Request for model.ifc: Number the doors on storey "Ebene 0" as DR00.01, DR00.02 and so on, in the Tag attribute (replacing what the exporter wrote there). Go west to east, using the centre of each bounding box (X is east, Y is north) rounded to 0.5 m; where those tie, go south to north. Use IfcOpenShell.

First a look at what the model holds.

```python
import ifcopenshell
import ifcopenshell.util.element
import ifcopenshell.util.placement

model = ifcopenshell.open("model.ifc")
print(model.schema)
storey = next(s for s in model.by_type("IfcBuildingStorey") if s.Name == "Ebene 0")
doors = [e for e in ifcopenshell.util.element.get_decomposition(storey) if e.is_a("IfcDoor")]
for e in sorted(doors, key=lambda e: e.id()):
    origin = ifcopenshell.util.placement.get_local_placement(e.ObjectPlacement)[:3, 3]
    print(e.id(), e.Tag, e.Name, origin.round(2) + 0.0, sep=" | ")
```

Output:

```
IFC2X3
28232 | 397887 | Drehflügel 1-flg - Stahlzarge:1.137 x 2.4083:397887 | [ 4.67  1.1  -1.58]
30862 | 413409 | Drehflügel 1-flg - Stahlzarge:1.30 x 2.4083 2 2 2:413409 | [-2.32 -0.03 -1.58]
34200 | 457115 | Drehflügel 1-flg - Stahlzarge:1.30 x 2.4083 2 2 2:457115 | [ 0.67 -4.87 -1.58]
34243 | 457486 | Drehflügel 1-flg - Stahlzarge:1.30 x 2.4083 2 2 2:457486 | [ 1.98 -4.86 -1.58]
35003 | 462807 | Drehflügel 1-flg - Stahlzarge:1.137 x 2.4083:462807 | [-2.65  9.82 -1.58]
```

```python
import ifcopenshell
import ifcopenshell.geom
import ifcopenshell.util.element
import ifcopenshell.util.shape

model = ifcopenshell.open("model.ifc")
settings = ifcopenshell.geom.settings()
settings.set("use-world-coords", True)


def centre(element):
    shape = ifcopenshell.geom.create_shape(settings, element)
    return ifcopenshell.util.shape.get_bbox_centroid(shape.geometry)


storey = next(s for s in model.by_type("IfcBuildingStorey") if s.Name == "Ebene 0")
doors = [e for e in ifcopenshell.util.element.get_decomposition(storey) if e.is_a("IfcDoor")]

# Insertion points can sit at a corner or the storey origin, so sort by the geometry (in metres).
centres = {e: centre(e) for e in doors}
doors.sort(key=lambda e: (round(centres[e][0] / 0.5), centres[e][1]))

for i, e in enumerate(doors, start=1):
    number = f"DR00.{i:02d}"
    e.Tag = number
    print(e.id(), number)

model.write("model_v2.ifc")
```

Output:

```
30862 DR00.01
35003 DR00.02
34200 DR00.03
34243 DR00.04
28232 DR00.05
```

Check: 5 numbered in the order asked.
